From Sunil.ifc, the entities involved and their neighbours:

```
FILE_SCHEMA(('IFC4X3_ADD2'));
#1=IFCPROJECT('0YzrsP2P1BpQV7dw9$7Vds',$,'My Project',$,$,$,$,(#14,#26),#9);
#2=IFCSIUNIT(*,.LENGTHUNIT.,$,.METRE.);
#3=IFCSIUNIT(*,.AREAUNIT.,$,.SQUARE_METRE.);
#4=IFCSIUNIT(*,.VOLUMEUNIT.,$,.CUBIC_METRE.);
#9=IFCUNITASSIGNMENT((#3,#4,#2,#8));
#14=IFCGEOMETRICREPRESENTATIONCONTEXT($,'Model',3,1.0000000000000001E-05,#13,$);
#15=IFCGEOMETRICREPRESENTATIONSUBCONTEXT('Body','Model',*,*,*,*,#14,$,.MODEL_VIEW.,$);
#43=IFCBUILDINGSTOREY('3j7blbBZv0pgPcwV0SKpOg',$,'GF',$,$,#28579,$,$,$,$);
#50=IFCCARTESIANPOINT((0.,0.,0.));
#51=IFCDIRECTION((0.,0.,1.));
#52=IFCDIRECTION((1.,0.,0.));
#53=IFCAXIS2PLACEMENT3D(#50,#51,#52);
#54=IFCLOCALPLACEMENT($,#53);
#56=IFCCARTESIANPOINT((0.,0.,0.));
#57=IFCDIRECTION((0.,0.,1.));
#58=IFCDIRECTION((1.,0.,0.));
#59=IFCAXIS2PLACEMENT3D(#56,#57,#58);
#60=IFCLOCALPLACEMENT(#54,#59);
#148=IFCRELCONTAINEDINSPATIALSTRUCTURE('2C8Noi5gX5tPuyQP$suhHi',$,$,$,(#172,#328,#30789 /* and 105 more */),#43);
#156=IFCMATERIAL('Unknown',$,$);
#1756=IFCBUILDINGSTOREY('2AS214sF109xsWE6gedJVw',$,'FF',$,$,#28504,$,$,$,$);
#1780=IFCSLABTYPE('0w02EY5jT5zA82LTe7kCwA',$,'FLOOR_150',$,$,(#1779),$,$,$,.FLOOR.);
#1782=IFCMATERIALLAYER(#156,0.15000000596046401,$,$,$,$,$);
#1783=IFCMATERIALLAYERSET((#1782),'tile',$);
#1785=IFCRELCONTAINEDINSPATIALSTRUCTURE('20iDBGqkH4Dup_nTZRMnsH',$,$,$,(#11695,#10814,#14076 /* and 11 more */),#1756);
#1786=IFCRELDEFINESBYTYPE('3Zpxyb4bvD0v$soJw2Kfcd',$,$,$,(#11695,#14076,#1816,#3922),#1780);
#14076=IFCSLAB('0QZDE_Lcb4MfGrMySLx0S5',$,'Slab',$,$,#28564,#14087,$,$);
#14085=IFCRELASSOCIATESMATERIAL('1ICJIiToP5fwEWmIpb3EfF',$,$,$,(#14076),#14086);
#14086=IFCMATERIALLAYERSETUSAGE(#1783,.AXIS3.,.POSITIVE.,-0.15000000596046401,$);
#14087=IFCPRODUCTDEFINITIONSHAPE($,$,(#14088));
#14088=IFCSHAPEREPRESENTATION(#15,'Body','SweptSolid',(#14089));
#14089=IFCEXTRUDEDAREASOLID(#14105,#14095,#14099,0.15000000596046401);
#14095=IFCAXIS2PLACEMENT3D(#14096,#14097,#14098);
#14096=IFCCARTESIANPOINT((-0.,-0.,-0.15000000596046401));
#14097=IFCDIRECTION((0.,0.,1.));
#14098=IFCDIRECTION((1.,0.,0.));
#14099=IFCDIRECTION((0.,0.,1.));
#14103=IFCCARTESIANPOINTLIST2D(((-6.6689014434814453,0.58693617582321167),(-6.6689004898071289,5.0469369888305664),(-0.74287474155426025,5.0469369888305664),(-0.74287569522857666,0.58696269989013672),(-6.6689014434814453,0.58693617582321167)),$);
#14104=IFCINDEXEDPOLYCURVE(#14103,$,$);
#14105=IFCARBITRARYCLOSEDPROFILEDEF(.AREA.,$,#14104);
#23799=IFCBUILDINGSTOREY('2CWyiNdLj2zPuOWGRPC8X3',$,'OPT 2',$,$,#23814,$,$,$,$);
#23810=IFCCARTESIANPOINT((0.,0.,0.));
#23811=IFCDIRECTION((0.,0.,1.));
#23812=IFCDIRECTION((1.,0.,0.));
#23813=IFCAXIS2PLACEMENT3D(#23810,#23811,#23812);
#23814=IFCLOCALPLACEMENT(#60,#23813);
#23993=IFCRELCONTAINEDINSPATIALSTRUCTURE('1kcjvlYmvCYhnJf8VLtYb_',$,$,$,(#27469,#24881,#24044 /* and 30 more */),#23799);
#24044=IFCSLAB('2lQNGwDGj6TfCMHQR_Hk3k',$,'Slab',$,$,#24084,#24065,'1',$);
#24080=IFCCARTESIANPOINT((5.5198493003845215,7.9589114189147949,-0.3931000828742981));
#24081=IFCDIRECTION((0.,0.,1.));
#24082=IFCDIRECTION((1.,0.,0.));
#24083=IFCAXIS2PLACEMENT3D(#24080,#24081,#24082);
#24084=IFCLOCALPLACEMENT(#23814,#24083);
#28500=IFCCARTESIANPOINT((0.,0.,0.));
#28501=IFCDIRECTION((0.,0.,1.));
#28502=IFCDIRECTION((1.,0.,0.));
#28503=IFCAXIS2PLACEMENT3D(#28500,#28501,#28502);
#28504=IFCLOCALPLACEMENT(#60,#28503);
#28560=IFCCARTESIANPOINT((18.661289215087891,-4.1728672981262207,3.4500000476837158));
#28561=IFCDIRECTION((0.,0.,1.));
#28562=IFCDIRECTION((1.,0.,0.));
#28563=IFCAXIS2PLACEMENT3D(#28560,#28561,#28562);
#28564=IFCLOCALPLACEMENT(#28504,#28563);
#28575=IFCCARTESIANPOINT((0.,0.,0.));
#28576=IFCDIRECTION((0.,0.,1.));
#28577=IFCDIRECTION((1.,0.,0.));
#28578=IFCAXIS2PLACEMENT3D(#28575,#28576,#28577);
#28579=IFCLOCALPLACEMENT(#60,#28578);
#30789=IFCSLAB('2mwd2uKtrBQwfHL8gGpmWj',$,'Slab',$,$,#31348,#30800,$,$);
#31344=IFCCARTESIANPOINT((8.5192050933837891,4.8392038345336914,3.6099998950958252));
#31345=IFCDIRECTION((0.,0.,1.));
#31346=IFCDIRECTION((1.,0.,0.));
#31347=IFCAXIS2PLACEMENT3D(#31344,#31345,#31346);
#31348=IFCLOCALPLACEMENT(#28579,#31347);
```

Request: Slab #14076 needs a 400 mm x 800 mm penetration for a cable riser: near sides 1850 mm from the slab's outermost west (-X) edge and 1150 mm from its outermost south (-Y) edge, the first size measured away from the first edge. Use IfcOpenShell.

```python
import numpy as np
import ifcopenshell
import ifcopenshell.api.feature
import ifcopenshell.api.geometry
import ifcopenshell.api.root
import ifcopenshell.geom
import ifcopenshell.util.placement
import ifcopenshell.util.representation
import ifcopenshell.util.shape
import ifcopenshell.util.unit

model = ifcopenshell.open("Sunil.ifc")
unit_scale = ifcopenshell.util.unit.calculate_unit_scale(model)
settings = ifcopenshell.geom.settings()


def volume(element):
    """Net volume in cubic metres, openings subtracted."""
    shape = ifcopenshell.geom.create_shape(settings, element)
    return ifcopenshell.util.shape.get_volume(shape.geometry)


slab = model.by_guid("0QZDE_Lcb4MfGrMySLx0S5")
before = volume(slab)

# Extent in the slab's own axes, in metres. The edges named are its -X and -Y sides.
slab_shape = ifcopenshell.geom.create_shape(settings, slab)
vertices = ifcopenshell.util.shape.get_vertices(slab_shape.geometry)
x_min, y_min, bottom = vertices.min(axis=0)
top = vertices[:, 2].max()

opening = ifcopenshell.api.root.create_entity(model, ifc_class="IfcOpeningElement", name="Cable riser opening", predefined_type="OPENING")
context = ifcopenshell.util.representation.get_context(model, "Model", "Body", "MODEL_VIEW")
width, depth = 0.4, 0.8
outline = [(0.0, 0.0), (width, 0.0), (width, depth), (0.0, depth), (0.0, 0.0)]
# Overshoot both faces by 50 mm so the cut is clean.
shape = ifcopenshell.api.geometry.add_slab_representation(
    model, context=context, depth=top - bottom + 0.1, polyline=outline
)
ifcopenshell.api.geometry.assign_representation(model, product=opening, representation=shape)

matrix = ifcopenshell.util.placement.get_local_placement(slab.ObjectPlacement)
matrix[:, 3] = matrix @ np.append(np.array([x_min + 1.85, y_min + 1.15, bottom - 0.05]) / unit_scale, 1.0)
ifcopenshell.api.geometry.edit_object_placement(model, product=opening, matrix=matrix, is_si=False)
ifcopenshell.api.feature.add_feature(model, feature=opening, element=slab)

after = volume(slab)

print(f"slab volume {before:.3f} -> {after:.3f} m3")

model.write("Sunil_edited.ifc")
```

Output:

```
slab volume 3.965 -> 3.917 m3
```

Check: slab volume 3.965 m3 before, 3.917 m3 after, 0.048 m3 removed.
